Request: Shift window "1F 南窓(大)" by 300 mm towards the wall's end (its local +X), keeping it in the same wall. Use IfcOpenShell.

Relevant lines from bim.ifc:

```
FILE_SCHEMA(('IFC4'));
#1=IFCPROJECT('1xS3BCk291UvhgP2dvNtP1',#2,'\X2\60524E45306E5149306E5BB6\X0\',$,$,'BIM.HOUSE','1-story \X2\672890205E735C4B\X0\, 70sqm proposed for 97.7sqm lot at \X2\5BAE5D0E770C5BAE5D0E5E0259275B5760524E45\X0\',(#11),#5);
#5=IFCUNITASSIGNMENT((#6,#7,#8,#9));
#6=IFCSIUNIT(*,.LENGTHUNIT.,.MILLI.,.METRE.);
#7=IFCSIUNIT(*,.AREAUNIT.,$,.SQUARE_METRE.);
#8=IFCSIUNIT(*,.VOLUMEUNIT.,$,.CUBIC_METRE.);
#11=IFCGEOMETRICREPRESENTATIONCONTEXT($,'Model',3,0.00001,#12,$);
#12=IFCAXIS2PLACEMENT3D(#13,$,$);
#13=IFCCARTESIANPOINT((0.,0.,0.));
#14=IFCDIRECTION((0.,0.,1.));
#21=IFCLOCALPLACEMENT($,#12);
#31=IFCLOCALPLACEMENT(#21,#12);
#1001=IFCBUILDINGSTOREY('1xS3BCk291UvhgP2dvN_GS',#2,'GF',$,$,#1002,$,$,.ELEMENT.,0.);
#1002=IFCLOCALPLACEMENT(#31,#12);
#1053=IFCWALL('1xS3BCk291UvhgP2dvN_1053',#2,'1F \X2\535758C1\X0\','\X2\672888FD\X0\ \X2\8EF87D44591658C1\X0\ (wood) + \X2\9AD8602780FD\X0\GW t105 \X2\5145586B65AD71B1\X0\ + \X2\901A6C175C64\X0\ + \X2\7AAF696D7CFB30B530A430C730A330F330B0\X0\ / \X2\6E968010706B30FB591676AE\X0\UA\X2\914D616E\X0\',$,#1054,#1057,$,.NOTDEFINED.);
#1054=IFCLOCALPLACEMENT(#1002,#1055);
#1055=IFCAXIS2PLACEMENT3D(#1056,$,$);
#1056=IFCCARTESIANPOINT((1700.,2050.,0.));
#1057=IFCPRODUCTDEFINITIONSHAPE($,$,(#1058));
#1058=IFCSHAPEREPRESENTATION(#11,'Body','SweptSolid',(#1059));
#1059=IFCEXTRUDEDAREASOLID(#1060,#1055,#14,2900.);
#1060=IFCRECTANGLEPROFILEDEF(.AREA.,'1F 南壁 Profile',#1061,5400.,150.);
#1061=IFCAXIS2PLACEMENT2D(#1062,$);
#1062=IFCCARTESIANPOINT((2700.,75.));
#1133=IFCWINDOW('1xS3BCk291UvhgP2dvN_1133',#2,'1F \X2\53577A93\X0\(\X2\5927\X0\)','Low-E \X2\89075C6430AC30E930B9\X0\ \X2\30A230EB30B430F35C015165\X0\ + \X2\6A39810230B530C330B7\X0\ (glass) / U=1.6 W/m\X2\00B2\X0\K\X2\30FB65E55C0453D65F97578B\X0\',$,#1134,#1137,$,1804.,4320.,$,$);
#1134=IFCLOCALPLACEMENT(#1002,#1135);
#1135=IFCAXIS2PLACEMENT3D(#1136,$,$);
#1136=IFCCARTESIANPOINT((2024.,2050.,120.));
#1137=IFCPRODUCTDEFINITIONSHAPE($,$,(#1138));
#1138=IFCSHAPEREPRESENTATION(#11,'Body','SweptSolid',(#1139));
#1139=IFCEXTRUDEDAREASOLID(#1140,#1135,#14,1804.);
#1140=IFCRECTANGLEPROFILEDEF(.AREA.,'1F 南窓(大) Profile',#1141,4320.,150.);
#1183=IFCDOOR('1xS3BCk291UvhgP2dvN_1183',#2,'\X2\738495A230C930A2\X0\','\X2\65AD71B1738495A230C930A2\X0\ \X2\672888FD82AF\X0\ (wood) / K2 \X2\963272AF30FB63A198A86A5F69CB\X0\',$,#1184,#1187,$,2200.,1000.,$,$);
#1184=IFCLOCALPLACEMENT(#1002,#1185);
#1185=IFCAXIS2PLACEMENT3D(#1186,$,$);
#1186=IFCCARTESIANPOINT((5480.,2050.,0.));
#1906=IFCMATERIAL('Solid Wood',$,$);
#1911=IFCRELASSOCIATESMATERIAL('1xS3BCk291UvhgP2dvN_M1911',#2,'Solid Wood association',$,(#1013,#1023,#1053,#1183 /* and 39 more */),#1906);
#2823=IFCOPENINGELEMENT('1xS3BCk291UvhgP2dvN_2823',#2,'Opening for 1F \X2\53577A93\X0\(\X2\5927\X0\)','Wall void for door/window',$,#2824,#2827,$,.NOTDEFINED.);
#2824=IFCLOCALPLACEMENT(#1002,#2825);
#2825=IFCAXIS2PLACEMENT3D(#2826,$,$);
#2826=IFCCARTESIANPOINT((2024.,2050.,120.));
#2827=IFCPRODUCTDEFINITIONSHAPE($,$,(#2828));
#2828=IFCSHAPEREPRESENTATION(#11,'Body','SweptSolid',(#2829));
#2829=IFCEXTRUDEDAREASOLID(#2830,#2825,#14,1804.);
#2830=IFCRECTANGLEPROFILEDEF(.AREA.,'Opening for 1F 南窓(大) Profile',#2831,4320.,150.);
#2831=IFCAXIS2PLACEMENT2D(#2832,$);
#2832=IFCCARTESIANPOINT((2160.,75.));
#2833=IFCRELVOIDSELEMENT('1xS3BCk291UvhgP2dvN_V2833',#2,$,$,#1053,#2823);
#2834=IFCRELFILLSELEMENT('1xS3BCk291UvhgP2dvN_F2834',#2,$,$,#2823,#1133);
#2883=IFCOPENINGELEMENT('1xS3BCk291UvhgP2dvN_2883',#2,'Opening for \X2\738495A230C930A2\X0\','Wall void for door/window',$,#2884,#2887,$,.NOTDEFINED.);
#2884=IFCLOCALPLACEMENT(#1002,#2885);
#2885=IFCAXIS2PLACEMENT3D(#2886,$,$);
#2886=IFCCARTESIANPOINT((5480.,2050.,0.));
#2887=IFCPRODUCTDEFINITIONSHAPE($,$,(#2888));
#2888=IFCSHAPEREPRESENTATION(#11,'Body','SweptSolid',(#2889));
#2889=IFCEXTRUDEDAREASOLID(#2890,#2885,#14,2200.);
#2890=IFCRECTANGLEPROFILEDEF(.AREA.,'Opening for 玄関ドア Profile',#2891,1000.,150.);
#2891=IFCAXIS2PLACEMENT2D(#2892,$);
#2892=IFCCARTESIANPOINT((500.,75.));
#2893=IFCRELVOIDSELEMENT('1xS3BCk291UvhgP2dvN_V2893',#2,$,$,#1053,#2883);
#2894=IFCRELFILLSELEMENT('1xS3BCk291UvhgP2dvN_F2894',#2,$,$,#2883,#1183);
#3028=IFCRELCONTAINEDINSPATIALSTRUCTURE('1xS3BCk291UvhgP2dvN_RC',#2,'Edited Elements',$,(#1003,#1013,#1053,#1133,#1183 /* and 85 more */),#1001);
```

```python
import ifcopenshell
import ifcopenshell.api.geometry
import ifcopenshell.util.placement

model = ifcopenshell.open("bim.ifc")

window = model.by_id(1133)
opening = window.FillsVoids[0].RelatingOpeningElement
wall = opening.VoidsElements[0].RelatingBuildingElement

wall_matrix = ifcopenshell.util.placement.get_local_placement(wall.ObjectPlacement)
shift = wall_matrix[:3, 0] * 300.0
before = ifcopenshell.util.placement.get_local_placement(window.ObjectPlacement)[:3, 3].copy()

# The window is not placed relative to its opening, so move both.
for product in (opening, window):
    matrix = ifcopenshell.util.placement.get_local_placement(product.ObjectPlacement)
    matrix[:3, 3] += shift
    ifcopenshell.api.geometry.edit_object_placement(model, product=product, matrix=matrix, is_si=False)

after = ifcopenshell.util.placement.get_local_placement(window.ObjectPlacement)[:3, 3]
print("window moved by", (after - before).round(3) + 0.0)

model.write("bim-out.ifc")
```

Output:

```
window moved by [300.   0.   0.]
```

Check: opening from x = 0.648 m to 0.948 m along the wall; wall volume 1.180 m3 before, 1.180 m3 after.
